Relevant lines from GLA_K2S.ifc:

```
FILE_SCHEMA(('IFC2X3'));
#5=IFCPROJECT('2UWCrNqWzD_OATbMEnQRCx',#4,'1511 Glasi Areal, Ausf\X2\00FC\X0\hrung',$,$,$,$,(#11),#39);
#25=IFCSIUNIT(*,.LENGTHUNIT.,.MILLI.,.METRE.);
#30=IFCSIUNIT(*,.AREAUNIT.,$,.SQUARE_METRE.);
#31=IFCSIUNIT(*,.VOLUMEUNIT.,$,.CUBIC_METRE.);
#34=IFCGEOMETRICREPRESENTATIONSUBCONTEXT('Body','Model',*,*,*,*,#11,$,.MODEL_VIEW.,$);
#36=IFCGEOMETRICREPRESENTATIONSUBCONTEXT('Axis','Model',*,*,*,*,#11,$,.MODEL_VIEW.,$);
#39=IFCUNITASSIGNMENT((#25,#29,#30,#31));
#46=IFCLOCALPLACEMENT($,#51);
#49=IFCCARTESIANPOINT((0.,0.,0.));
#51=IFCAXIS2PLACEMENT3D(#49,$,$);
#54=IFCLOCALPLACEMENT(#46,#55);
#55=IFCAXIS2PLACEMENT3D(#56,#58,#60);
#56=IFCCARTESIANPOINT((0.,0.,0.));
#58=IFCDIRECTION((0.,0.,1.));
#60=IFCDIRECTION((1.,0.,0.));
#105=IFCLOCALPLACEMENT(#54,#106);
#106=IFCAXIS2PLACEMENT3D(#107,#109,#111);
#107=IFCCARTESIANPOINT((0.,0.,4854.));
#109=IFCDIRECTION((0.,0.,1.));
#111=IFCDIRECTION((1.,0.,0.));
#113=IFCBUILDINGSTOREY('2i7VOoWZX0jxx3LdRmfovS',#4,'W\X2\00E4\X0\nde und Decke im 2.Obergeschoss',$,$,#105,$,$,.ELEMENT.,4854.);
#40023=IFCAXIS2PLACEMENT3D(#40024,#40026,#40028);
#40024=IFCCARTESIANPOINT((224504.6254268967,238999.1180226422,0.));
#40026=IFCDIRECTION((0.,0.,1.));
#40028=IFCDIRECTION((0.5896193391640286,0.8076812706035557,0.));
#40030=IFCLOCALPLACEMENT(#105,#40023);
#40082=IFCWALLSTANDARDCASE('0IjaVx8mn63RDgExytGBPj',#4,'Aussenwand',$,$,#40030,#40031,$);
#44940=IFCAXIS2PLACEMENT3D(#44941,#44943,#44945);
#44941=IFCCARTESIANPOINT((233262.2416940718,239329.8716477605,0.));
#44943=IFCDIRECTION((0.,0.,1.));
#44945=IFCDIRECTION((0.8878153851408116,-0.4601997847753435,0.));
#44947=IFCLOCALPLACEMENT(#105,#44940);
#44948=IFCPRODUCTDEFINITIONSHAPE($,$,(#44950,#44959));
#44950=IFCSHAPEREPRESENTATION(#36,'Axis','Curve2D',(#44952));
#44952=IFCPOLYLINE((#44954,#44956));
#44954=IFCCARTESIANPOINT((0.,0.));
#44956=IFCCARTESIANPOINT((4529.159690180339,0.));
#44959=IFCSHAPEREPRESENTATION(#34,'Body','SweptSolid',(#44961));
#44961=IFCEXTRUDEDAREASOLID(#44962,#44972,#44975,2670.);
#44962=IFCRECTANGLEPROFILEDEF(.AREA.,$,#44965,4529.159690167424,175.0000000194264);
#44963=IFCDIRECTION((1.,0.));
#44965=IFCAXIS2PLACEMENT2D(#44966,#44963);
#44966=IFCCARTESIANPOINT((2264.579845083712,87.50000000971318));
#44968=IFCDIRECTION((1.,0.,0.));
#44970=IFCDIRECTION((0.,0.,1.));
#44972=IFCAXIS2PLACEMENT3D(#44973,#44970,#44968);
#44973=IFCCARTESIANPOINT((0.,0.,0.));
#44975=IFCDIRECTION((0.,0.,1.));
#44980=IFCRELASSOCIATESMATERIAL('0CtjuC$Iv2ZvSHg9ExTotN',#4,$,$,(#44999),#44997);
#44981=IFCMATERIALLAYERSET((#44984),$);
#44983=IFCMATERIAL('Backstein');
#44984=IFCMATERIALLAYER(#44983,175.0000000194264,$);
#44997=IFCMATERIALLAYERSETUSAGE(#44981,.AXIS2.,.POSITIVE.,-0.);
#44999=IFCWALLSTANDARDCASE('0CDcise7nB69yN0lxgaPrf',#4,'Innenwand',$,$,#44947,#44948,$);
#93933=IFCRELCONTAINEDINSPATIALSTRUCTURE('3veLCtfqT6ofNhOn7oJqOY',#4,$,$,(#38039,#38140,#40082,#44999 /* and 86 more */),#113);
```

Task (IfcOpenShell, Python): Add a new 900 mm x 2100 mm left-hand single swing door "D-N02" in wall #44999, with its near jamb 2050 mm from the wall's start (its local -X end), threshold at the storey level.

```python
import numpy as np
import ifcopenshell
import ifcopenshell.api.feature
import ifcopenshell.api.geometry
import ifcopenshell.api.root
import ifcopenshell.api.spatial
import ifcopenshell.api.type
import ifcopenshell.geom
import ifcopenshell.util.element
import ifcopenshell.util.placement
import ifcopenshell.util.representation
import ifcopenshell.util.shape
import ifcopenshell.util.unit

model = ifcopenshell.open("GLA_K2S.ifc")
unit_scale = ifcopenshell.util.unit.calculate_unit_scale(model)
settings = ifcopenshell.geom.settings()


def volume(element):
    """Net volume in cubic metres, openings subtracted."""
    shape = ifcopenshell.geom.create_shape(settings, element)
    return ifcopenshell.util.shape.get_volume(shape.geometry)


wall = model.by_guid("0CDcise7nB69yN0lxgaPrf")
storey = ifcopenshell.util.element.get_container(wall, ifc_class="IfcBuildingStorey")
context = ifcopenshell.util.representation.get_context(model, "Model", "Body", "MODEL_VIEW")
before = volume(wall)

width, height, from_end, sill = 0.9, 2.1, 2.05, 0.0  # metres

# The wall runs along its own X axis, and the end named is its -X end.
wall_shape = ifcopenshell.geom.create_shape(settings, wall)
x, y, z = ifcopenshell.util.shape.get_vertices(wall_shape.geometry).T
start = x.min() + from_end
face, thickness = float(y.min()), float(y.max() - y.min())
wall_matrix = ifcopenshell.util.placement.get_local_placement(wall.ObjectPlacement)
level = ifcopenshell.util.placement.get_local_placement(storey.ObjectPlacement)[2, 3]


def in_wall(x, y):
    """Placement at x, y metres in the wall's axes, at sill height."""
    matrix = wall_matrix.copy()
    matrix[:, 3] = wall_matrix @ np.array([x / unit_scale, y / unit_scale, 0.0, 1.0])
    matrix[2, 3] = level + sill / unit_scale
    return matrix


# Opening: a box that overshoots both wall faces by 50 mm.
opening = ifcopenshell.api.root.create_entity(model, ifc_class="IfcOpeningElement")
box = ifcopenshell.api.geometry.add_wall_representation(
    model, context=context, length=width, height=height, thickness=thickness + 0.1
)
ifcopenshell.api.geometry.assign_representation(model, product=opening, representation=box)
ifcopenshell.api.geometry.edit_object_placement(model, product=opening, matrix=in_wall(start, face - 0.05), is_si=False)
ifcopenshell.api.feature.add_feature(model, feature=opening, element=wall)

door = ifcopenshell.api.root.create_entity(model, ifc_class="IfcDoor", name="D-N02")
door.OverallWidth, door.OverallHeight = width / unit_scale, height / unit_scale
body = ifcopenshell.api.geometry.add_door_representation(
    model,
    context=context,
    overall_width=door.OverallWidth,
    overall_height=door.OverallHeight,
    operation_type="SINGLE_SWING_LEFT",
    lining_properties={"LiningDepth": thickness / unit_scale, "ThresholdDepth": thickness / unit_scale},
)
ifcopenshell.api.geometry.assign_representation(model, product=door, representation=body)
ifcopenshell.api.spatial.assign_container(model, products=[door], relating_structure=storey)
fills = ifcopenshell.api.feature.add_filling(model, opening=opening, element=door)
fills.OwnerHistory = door.OwnerHistory  # required in IFC2X3

# IFC2X3 keeps the operation on the door style.
style = ifcopenshell.api.root.create_entity(model, ifc_class="IfcDoorStyle", name="D-N02")
style.OperationType, style.ConstructionType = "SINGLE_SWING_LEFT", "NOTDEFINED"
style.ParameterTakesPrecedence = style.Sizeable = False
ifcopenshell.api.type.assign_type(model, related_objects=[door], relating_type=style)

# The lining spans the wall, so the door starts at the wall face.
ifcopenshell.api.geometry.edit_object_placement(model, product=door, matrix=in_wall(start, face), is_si=False)

after = volume(wall)

print(f"wall volume {before:.3f} -> {after:.3f} m3")

model.write("GLA_K2S-out.ifc")
```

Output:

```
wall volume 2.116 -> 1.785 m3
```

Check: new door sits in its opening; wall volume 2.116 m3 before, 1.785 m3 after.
